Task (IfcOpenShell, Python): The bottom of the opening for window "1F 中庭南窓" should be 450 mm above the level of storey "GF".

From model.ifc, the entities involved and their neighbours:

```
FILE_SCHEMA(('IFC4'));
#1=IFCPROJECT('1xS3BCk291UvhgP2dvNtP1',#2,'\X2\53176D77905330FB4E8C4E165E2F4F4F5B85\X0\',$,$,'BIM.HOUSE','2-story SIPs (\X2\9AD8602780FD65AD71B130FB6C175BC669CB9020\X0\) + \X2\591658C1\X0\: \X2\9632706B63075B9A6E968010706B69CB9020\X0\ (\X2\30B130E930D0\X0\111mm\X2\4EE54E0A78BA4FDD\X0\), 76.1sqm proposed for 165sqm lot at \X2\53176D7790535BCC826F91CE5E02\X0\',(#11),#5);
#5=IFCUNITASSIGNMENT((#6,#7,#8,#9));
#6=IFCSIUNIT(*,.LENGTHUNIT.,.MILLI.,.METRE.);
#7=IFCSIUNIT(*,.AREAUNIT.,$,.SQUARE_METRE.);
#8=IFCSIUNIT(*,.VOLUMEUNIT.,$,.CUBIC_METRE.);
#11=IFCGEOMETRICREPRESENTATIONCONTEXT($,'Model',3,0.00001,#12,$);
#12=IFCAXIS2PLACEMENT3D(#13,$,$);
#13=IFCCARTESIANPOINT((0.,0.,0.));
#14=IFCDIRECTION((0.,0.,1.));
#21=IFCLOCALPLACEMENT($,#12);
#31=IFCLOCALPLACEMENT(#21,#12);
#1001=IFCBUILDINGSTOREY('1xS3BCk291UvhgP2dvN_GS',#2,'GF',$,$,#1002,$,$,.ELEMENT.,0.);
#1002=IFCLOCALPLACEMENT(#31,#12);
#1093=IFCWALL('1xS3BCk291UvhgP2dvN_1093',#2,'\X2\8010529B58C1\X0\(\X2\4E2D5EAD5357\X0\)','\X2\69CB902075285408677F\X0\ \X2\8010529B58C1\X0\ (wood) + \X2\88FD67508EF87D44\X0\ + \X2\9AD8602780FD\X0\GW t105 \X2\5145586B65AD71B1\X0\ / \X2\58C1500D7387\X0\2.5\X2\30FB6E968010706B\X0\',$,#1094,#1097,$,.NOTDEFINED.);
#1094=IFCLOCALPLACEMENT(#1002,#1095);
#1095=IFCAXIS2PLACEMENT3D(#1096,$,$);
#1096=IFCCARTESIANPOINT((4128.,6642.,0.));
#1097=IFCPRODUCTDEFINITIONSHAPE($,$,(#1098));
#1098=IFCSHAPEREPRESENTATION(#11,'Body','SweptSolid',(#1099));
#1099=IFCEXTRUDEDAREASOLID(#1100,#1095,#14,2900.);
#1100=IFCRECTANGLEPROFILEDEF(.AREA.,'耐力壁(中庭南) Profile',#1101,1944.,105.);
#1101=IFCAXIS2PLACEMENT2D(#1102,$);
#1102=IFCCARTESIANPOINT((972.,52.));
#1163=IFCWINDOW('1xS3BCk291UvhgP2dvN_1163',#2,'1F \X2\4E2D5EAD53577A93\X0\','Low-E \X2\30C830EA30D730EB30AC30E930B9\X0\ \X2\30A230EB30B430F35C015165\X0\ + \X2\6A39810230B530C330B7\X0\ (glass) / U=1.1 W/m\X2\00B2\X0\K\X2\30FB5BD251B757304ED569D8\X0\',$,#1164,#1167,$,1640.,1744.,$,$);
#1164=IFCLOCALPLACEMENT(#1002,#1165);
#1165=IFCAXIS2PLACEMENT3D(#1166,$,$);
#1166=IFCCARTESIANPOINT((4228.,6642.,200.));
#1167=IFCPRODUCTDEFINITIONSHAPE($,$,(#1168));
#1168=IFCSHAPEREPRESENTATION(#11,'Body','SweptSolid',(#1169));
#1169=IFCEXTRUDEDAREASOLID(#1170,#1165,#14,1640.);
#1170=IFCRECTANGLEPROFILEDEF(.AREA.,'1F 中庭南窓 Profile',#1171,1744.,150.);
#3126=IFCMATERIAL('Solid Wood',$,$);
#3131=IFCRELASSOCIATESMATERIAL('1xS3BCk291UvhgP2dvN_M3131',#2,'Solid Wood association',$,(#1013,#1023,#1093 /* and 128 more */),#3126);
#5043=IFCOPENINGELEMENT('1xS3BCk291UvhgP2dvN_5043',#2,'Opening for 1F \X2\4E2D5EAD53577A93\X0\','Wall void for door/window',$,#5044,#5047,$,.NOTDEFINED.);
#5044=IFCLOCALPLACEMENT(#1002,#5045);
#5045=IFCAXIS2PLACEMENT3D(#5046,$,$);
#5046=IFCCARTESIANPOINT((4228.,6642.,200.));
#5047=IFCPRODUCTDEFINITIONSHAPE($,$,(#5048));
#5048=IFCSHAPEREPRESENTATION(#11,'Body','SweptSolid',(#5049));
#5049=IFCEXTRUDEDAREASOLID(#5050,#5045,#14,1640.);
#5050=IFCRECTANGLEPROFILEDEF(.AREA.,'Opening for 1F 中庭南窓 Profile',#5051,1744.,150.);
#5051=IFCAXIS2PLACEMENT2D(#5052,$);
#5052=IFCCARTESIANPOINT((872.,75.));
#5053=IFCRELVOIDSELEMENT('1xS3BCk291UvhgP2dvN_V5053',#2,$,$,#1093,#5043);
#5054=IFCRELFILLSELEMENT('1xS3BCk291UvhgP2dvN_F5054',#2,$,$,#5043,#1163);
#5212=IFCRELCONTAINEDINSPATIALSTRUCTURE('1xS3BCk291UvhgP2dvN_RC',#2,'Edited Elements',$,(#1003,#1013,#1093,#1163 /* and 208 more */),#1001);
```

```python
import numpy as np
import ifcopenshell
import ifcopenshell.api.geometry
import ifcopenshell.geom
import ifcopenshell.util.element
import ifcopenshell.util.placement
import ifcopenshell.util.shape
import ifcopenshell.util.unit

model = ifcopenshell.open("model.ifc")
unit_scale = ifcopenshell.util.unit.calculate_unit_scale(model)

window = model.by_guid("1xS3BCk291UvhgP2dvN_1163")
opening = window.FillsVoids[0].RelatingOpeningElement
storey = ifcopenshell.util.element.get_container(window, ifc_class="IfcBuildingStorey")
level = ifcopenshell.util.placement.get_local_placement(storey.ObjectPlacement)[2, 3]

# The opening's origin need not be at the sill, so measure its lowest point.
shape = ifcopenshell.geom.create_shape(ifcopenshell.geom.settings(), opening)
bottom = ifcopenshell.util.shape.get_shape_bottom_elevation(shape, shape.geometry) / unit_scale
dz = level + 0.45 / unit_scale - bottom

shift = np.array([0.0, 0.0, dz])
# The window is not placed relative to its opening, so move both.
for product in (opening, window):
    matrix = ifcopenshell.util.placement.get_local_placement(product.ObjectPlacement)
    matrix[:3, 3] += shift
    ifcopenshell.api.geometry.edit_object_placement(model, product=product, matrix=matrix, is_si=False)

print(f"moved by {dz * unit_scale:+.3f} m")

model.write("model_updated.ifc")
```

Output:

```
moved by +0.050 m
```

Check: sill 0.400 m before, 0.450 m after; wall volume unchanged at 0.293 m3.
